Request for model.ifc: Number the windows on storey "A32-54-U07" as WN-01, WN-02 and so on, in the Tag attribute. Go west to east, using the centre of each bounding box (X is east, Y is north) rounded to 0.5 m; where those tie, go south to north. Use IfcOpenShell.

First a look at what the model holds.

```python
import ifcopenshell
import ifcopenshell.util.element
import ifcopenshell.util.placement

model = ifcopenshell.open("model.ifc")
print(model.schema)
storey = next(s for s in model.by_type("IfcBuildingStorey") if s.Name == "A32-54-U07")
windows = [e for e in ifcopenshell.util.element.get_decomposition(storey) if e.is_a("IfcWindow")]
for e in sorted(windows, key=lambda e: e.id()):
    origin = ifcopenshell.util.placement.get_local_placement(e.ObjectPlacement)[:3, 3]
    print(e.id(), e.Tag, e.Name, origin.round(2) + 0.0, sep=" | ")
```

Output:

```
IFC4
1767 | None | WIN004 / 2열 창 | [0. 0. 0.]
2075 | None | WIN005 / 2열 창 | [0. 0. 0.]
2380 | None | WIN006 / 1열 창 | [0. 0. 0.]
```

```python
import ifcopenshell
import ifcopenshell.geom
import ifcopenshell.util.element
import ifcopenshell.util.shape

model = ifcopenshell.open("model.ifc")
settings = ifcopenshell.geom.settings()
settings.set("use-world-coords", True)


def centre(element):
    shape = ifcopenshell.geom.create_shape(settings, element)
    return ifcopenshell.util.shape.get_bbox_centroid(shape.geometry)


storey = next(s for s in model.by_type("IfcBuildingStorey") if s.Name == "A32-54-U07")
windows = [e for e in ifcopenshell.util.element.get_decomposition(storey) if e.is_a("IfcWindow")]

# Insertion points can sit at a corner or the storey origin, so sort by the geometry (in metres).
centres = {e: centre(e) for e in windows}
windows.sort(key=lambda e: (round(centres[e][0] / 0.5), centres[e][1]))

for i, e in enumerate(windows, start=1):
    number = f"WN-{i:02d}"
    e.Tag = number
    print(e.id(), number)

model.write("model-out.ifc")
```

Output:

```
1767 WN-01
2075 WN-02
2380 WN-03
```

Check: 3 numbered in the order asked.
